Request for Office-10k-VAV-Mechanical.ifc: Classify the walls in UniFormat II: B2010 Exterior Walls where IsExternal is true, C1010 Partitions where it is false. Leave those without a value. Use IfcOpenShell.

First a look at what the model holds.

```python
import ifcopenshell
import ifcopenshell.util.element

model = ifcopenshell.open("Office-10k-VAV-Mechanical.ifc")
print(model.schema)
print("classifications:", [c.Name for c in model.by_type("IfcClassification")])
values = [ifcopenshell.util.element.get_pset(e, "Pset_WallCommon", "IsExternal") for e in model.by_type("IfcWall")]
for value in (True, False, None):
    print("IsExternal", value, values.count(value))
```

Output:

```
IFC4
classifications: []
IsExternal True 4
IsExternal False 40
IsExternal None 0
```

```python
import ifcopenshell
import ifcopenshell.api.classification
import ifcopenshell.util.element

model = ifcopenshell.open("Office-10k-VAV-Mechanical.ifc")

system = ifcopenshell.api.classification.add_classification(model, classification="UniFormat II")

walls = model.by_type("IfcWall")
external = {e: ifcopenshell.util.element.get_pset(e, "Pset_WallCommon", "IsExternal") for e in walls}
for flag, code, name in ((True, "B2010", "Exterior Walls"), (False, "C1010", "Partitions")):
    products = [e for e in walls if external[e] is flag]
    ifcopenshell.api.classification.add_reference(
        model, products=products, classification=system, identification=code, name=name
    )
    print(code, len(products))

model.write("Office-10k-VAV-Mechanical_v2.ifc")
```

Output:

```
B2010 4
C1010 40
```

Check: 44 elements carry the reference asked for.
